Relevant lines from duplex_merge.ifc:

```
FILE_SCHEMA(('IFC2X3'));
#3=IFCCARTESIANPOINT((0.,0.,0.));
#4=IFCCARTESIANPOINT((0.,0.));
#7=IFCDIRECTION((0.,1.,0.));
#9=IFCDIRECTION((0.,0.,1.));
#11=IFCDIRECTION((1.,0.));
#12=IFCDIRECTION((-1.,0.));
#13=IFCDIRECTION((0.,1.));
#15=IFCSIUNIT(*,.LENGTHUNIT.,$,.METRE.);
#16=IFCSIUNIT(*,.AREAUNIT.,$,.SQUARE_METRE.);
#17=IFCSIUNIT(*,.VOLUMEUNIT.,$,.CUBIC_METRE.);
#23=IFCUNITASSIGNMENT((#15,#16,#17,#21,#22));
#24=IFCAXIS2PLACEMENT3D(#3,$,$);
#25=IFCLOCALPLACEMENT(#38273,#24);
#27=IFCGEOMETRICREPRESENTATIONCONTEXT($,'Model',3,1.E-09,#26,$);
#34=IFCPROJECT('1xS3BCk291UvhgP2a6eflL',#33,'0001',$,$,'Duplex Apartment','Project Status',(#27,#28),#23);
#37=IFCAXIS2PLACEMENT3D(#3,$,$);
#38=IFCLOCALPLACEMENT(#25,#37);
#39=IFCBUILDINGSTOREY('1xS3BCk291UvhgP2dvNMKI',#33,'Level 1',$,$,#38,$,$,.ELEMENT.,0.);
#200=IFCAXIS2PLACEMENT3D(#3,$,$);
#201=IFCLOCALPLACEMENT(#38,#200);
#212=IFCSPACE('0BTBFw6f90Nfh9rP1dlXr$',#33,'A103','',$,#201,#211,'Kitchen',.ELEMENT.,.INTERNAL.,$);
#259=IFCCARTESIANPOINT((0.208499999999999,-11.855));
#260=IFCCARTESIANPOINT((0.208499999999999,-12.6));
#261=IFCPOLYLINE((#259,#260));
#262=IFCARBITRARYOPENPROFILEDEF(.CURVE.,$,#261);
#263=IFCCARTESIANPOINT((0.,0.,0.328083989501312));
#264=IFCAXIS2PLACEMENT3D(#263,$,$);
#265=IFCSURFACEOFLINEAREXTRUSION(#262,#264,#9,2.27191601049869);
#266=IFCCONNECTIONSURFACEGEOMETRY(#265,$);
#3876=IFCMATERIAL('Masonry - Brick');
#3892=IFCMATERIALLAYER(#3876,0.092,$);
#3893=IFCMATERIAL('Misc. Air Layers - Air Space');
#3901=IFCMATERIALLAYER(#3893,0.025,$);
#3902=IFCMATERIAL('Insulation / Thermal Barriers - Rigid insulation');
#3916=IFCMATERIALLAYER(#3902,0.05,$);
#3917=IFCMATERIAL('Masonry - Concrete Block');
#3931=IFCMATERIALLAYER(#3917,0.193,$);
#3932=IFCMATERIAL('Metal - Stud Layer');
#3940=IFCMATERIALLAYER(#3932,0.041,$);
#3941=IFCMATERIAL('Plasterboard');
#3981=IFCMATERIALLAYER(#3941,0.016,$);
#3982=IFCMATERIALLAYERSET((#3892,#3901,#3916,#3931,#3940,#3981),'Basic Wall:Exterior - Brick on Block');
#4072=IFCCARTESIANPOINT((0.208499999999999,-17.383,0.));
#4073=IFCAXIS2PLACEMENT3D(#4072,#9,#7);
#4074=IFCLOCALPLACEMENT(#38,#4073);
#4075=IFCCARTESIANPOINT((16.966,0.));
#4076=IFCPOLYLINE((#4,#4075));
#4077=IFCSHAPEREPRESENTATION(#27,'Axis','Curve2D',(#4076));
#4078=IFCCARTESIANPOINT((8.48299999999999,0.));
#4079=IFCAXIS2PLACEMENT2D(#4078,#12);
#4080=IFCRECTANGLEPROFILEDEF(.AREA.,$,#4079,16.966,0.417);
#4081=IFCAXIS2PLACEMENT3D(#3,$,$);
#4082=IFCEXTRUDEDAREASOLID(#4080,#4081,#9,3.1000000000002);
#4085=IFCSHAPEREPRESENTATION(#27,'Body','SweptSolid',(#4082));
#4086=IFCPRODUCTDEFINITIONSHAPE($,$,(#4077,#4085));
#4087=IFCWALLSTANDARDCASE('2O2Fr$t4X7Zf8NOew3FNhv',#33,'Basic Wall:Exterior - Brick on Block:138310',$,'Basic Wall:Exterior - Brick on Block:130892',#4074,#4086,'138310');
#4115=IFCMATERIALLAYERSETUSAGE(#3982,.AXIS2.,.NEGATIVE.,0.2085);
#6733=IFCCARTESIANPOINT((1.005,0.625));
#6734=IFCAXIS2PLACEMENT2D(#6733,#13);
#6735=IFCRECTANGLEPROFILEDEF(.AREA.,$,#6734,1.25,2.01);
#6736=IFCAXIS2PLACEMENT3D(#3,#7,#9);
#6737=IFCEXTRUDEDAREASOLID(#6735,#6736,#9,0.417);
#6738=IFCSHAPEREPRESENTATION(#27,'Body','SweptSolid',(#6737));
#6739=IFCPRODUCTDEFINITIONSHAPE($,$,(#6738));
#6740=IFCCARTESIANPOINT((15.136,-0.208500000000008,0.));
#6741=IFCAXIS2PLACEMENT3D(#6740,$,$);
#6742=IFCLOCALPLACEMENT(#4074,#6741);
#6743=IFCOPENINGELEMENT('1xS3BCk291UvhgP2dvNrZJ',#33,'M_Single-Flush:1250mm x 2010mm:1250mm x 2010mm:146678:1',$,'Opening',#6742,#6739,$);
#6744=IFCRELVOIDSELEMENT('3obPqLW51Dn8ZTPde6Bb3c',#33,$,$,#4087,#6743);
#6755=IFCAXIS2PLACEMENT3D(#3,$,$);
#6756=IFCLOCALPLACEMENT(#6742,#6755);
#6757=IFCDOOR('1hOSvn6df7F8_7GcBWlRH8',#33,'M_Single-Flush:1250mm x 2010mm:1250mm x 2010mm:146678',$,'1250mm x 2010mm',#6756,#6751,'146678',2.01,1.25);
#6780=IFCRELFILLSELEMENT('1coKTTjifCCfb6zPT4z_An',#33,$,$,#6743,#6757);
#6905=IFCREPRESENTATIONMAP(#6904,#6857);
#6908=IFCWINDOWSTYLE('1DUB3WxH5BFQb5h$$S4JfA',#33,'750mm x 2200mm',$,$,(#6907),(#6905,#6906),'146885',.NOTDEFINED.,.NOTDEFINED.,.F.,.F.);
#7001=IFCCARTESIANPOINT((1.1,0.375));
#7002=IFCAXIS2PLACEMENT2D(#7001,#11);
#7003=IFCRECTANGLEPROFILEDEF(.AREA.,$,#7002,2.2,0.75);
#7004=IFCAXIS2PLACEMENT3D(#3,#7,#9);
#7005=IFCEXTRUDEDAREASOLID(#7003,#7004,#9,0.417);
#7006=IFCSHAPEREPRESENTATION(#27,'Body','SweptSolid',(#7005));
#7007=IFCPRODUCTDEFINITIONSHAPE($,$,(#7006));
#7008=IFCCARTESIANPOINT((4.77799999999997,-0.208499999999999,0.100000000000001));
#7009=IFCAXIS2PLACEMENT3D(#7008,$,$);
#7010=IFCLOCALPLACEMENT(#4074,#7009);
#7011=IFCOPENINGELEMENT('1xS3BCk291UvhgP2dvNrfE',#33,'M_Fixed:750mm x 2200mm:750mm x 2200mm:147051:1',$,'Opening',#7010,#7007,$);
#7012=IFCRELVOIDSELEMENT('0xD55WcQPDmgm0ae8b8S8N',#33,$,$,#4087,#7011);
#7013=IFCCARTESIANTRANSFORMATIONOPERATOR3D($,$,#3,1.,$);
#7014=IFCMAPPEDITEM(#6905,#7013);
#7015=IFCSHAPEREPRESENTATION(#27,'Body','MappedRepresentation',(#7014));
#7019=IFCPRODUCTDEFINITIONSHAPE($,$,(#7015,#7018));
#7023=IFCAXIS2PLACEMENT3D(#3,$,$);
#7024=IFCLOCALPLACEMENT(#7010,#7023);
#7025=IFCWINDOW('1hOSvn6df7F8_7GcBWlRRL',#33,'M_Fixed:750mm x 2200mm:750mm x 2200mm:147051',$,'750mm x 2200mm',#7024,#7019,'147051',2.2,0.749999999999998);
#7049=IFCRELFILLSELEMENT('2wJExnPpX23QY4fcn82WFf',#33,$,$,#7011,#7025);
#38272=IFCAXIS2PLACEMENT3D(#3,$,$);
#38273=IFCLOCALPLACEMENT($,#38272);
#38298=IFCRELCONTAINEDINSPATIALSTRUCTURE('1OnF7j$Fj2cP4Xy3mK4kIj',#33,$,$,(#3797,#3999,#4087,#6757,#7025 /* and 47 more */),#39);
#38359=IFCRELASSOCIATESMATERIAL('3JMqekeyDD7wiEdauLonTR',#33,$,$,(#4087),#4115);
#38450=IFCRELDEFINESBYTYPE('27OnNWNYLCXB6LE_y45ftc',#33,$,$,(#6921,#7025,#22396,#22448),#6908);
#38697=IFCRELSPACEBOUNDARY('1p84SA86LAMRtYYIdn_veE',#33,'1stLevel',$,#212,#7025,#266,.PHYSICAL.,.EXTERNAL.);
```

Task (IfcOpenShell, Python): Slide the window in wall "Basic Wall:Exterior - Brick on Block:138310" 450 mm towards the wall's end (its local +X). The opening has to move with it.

```python
import numpy as np
import ifcopenshell
import ifcopenshell.api.geometry
import ifcopenshell.util.placement

model = ifcopenshell.open("duplex_merge.ifc")

window = model.by_guid("1hOSvn6df7F8_7GcBWlRRL")
opening = window.FillsVoids[0].RelatingOpeningElement
wall = opening.VoidsElements[0].RelatingBuildingElement

wall_matrix = ifcopenshell.util.placement.get_local_placement(wall.ObjectPlacement)
shift = wall_matrix[:3, 0] * 0.45
before = ifcopenshell.util.placement.get_local_placement(window.ObjectPlacement)[:3, 3].copy()

# The window is placed relative to its opening, so it follows when the opening moves.
matrix = ifcopenshell.util.placement.get_local_placement(opening.ObjectPlacement)
matrix[:3, 3] += shift
ifcopenshell.api.geometry.edit_object_placement(
    model, product=opening, matrix=matrix, is_si=False, should_transform_children=True
)

# Space boundary surfaces are stored in each space's coordinates; move them too.
for rel in window.ProvidesBoundaries:
    if not rel.ConnectionGeometry:
        continue
    surface = rel.ConnectionGeometry.SurfaceOnRelatingElement
    space_matrix = ifcopenshell.util.placement.get_local_placement(rel.RelatingSpace.ObjectPlacement)
    point = np.array(surface.Position.Location.Coordinates) + space_matrix[:3, :3].T @ shift
    surface.Position = model.createIfcAxis2Placement3D(
        model.createIfcCartesianPoint(point.tolist()), surface.Position.Axis, surface.Position.RefDirection
    )

after = ifcopenshell.util.placement.get_local_placement(window.ObjectPlacement)[:3, 3]
print("window moved by", (after - before).round(3) + 0.0)

model.write("duplex_merge_v2.ifc")
```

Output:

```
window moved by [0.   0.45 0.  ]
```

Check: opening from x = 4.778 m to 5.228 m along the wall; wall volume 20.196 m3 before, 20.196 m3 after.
